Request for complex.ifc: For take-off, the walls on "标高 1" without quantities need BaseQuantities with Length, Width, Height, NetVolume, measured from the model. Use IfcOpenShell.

First a look at what the model holds.

```python
import ifcopenshell
import ifcopenshell.util.element
import ifcopenshell.util.unit

model = ifcopenshell.open("complex.ifc")
print(model.schema)
for unit_type in ("LENGTHUNIT", "AREAUNIT", "VOLUMEUNIT"):
    print(unit_type, ifcopenshell.util.unit.calculate_unit_scale(model, unit_type))
storey = next(s for s in model.by_type("IfcBuildingStorey") if s.Name == "标高 1")
walls = [e for e in ifcopenshell.util.element.get_decomposition(storey) if e.is_a("IfcWall")]
for e in sorted(walls, key=lambda e: e.id()):
    print(e.id(), e.is_a(), e.Name, list(ifcopenshell.util.element.get_psets(e, qtos_only=True)), sep=" | ")
```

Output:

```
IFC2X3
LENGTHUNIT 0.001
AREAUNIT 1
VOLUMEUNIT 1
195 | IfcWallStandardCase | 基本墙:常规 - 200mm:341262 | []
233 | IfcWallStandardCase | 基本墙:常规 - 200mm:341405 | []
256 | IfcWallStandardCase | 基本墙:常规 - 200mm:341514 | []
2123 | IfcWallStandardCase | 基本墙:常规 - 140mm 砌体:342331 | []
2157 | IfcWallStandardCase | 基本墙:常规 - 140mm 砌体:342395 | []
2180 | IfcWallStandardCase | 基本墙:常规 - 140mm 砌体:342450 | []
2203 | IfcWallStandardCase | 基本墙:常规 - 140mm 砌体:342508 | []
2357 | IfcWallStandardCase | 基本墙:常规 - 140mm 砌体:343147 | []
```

```python
import ifcopenshell
import ifcopenshell.api.pset
import ifcopenshell.geom
import ifcopenshell.util.element
import ifcopenshell.util.shape
import ifcopenshell.util.unit

model = ifcopenshell.open("complex.ifc")
unit_scale = ifcopenshell.util.unit.calculate_unit_scale(model)
volume_scale = ifcopenshell.util.unit.calculate_unit_scale(model, "VOLUMEUNIT")
settings = ifcopenshell.geom.settings()

storey = next(s for s in model.by_type("IfcBuildingStorey") if s.Name == "标高 1")
walls = [e for e in ifcopenshell.util.element.get_decomposition(storey) if e.is_a("IfcWall")]

for e in sorted(walls, key=lambda e: e.id()):
    if ifcopenshell.util.element.get_psets(e, qtos_only=True, should_inherit=False):
        continue
    # Geometry comes back in metres, in the element's own axes.
    shape = ifcopenshell.geom.create_shape(settings, e)
    values = {
        "Length": ifcopenshell.util.shape.get_x(shape.geometry) / unit_scale,
        "Width": ifcopenshell.util.shape.get_y(shape.geometry) / unit_scale,
        "Height": ifcopenshell.util.shape.get_z(shape.geometry) / unit_scale,
        "NetVolume": ifcopenshell.util.shape.get_volume(shape.geometry) / volume_scale,
    }
    qto = ifcopenshell.api.pset.add_qto(model, product=e, name="BaseQuantities")
    ifcopenshell.api.pset.edit_qto(model, qto=qto, properties=values)
    print(e.id(), {k: round(v, 3) for k, v in values.items()})

model.write("complex_v2.ifc")
```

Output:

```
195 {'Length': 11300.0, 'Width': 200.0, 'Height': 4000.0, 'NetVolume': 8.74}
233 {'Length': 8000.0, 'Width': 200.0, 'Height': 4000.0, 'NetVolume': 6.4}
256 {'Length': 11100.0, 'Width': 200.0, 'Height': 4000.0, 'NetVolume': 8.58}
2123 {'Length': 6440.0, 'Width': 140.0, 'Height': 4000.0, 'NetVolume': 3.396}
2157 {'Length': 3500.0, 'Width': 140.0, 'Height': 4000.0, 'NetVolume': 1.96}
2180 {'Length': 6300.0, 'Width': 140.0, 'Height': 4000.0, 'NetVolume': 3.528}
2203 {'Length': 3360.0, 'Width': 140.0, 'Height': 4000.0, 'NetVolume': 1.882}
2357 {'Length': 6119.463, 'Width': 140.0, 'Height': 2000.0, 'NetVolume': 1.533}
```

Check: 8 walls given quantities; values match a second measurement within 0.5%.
